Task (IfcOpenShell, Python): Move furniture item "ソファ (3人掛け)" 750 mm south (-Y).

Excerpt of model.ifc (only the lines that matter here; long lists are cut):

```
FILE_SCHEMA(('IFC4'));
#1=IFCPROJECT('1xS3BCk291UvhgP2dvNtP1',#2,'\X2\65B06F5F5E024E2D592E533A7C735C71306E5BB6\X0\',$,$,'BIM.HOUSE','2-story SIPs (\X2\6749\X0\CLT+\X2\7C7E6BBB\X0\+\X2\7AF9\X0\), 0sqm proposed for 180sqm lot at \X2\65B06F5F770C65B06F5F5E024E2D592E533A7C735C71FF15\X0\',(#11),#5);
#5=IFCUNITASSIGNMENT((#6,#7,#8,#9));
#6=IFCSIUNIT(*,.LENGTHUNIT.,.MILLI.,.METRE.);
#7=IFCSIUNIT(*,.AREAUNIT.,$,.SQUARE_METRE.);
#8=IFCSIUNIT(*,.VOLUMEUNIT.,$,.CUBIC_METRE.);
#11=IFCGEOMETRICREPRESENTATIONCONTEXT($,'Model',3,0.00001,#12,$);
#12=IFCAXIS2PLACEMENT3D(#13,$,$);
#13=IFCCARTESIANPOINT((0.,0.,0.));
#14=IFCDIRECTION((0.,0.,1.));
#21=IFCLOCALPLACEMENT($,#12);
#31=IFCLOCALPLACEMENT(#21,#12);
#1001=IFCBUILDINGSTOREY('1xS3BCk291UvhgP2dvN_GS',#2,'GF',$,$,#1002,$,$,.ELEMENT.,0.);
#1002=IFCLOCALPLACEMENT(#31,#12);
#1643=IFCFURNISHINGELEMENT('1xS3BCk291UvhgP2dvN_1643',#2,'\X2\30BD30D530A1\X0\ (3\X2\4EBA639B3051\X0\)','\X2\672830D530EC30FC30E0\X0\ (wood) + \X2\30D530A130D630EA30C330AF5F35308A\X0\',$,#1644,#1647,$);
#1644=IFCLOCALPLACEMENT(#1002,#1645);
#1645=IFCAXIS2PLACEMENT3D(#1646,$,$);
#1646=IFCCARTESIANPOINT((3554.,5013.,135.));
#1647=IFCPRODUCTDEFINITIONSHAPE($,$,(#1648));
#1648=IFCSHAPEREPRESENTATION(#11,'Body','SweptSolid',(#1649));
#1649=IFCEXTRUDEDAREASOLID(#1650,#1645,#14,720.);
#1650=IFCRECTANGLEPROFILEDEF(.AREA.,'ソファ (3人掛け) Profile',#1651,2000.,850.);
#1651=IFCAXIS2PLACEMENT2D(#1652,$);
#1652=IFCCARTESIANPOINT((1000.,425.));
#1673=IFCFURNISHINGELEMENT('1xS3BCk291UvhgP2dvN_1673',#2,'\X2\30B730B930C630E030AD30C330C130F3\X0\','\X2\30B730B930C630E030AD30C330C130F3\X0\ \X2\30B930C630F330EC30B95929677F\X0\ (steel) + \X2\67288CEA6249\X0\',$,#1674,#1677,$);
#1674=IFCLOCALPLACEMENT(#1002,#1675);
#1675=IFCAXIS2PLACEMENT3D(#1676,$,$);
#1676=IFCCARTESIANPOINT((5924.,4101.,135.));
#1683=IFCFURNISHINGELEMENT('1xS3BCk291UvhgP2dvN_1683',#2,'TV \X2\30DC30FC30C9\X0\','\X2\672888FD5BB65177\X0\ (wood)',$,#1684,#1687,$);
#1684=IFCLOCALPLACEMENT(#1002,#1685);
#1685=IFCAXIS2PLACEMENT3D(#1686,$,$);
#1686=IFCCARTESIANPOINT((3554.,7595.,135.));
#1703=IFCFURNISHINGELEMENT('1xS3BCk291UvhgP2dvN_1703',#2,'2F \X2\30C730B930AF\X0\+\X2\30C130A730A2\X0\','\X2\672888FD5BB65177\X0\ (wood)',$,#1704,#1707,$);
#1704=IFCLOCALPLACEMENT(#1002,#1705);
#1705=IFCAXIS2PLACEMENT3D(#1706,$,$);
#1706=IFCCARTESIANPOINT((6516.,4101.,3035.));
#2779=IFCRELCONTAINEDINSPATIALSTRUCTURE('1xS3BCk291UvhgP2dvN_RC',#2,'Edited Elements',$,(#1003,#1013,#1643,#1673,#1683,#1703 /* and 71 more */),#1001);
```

```python
import ifcopenshell
import ifcopenshell.api.geometry
import ifcopenshell.util.placement
import ifcopenshell.util.unit

model = ifcopenshell.open("model.ifc")
unit_scale = ifcopenshell.util.unit.calculate_unit_scale(model)

item = model.by_guid("1xS3BCk291UvhgP2dvN_1643")
matrix = ifcopenshell.util.placement.get_local_placement(item.ObjectPlacement)
matrix[1, 3] -= 0.75 / unit_scale
ifcopenshell.api.geometry.edit_object_placement(model, product=item, matrix=matrix, is_si=False)

print(ifcopenshell.util.placement.get_local_placement(item.ObjectPlacement).round(3) + 0.0)

model.write("model_rev.ifc")
```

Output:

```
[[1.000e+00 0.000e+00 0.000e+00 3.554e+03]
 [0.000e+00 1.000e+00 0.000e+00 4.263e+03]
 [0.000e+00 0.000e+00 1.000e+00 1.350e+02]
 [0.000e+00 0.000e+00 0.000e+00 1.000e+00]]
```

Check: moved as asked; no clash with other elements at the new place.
